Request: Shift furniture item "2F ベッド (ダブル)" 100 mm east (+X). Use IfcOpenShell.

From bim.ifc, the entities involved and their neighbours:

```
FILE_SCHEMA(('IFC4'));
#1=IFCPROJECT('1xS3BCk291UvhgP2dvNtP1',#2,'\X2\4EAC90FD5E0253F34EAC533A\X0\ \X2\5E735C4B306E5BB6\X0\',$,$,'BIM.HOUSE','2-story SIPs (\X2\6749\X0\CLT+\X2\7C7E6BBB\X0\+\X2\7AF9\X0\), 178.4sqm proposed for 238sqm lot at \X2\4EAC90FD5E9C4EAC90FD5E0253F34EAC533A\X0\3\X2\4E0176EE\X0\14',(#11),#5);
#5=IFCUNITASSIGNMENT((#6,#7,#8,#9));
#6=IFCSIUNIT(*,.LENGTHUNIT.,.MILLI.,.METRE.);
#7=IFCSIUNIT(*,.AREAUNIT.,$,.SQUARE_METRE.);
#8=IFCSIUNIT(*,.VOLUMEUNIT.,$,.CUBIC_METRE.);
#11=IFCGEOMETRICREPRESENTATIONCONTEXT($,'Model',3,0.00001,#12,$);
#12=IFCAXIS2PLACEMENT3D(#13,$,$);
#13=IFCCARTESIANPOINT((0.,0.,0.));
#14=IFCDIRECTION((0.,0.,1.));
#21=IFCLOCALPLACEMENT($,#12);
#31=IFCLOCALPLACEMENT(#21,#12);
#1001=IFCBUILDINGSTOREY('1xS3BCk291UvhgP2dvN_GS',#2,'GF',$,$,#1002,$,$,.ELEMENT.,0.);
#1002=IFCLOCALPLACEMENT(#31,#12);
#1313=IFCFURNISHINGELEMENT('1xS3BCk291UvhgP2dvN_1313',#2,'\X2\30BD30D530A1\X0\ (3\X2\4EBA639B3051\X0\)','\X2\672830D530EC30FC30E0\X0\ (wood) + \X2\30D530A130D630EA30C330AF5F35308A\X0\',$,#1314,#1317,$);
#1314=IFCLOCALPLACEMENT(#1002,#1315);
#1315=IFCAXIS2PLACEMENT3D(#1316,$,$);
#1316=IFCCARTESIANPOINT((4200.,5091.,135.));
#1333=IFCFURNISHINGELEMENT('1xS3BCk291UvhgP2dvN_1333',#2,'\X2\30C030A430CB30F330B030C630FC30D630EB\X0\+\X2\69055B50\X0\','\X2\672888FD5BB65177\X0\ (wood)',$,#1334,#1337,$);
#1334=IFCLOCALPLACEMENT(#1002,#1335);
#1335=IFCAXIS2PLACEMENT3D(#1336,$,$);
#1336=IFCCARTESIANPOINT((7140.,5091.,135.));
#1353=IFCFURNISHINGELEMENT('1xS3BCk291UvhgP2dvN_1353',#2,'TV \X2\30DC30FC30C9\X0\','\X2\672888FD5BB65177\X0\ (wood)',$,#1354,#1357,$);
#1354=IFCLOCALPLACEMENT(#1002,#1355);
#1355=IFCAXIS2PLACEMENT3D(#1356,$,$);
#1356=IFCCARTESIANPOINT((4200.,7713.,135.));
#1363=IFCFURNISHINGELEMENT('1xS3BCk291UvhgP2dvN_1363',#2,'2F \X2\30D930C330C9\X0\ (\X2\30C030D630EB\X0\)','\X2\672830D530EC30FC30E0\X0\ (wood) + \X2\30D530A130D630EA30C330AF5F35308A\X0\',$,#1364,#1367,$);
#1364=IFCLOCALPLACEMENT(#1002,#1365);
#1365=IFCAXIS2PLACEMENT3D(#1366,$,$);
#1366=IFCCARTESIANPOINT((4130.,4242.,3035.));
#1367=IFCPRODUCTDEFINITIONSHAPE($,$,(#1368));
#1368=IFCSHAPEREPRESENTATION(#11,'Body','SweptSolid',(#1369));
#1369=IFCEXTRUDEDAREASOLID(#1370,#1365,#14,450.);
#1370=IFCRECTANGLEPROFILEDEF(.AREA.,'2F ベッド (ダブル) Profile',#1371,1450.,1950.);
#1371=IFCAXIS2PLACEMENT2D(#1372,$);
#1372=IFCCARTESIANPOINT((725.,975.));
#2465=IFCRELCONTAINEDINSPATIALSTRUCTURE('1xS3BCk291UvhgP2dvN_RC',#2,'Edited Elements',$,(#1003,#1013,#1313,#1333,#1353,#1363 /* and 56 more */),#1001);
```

```python
import ifcopenshell
import ifcopenshell.api.geometry
import ifcopenshell.util.placement
import ifcopenshell.util.unit

model = ifcopenshell.open("bim.ifc")
unit_scale = ifcopenshell.util.unit.calculate_unit_scale(model)

item = model.by_guid("1xS3BCk291UvhgP2dvN_1363")
matrix = ifcopenshell.util.placement.get_local_placement(item.ObjectPlacement)
matrix[0, 3] += 0.1 / unit_scale
ifcopenshell.api.geometry.edit_object_placement(model, product=item, matrix=matrix, is_si=False)

print(ifcopenshell.util.placement.get_local_placement(item.ObjectPlacement).round(3) + 0.0)

model.write("bim-out.ifc")
```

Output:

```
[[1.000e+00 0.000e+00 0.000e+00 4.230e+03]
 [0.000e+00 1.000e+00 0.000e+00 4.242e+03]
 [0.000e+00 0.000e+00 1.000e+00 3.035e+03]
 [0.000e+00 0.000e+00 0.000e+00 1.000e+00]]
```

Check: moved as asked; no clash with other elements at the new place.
